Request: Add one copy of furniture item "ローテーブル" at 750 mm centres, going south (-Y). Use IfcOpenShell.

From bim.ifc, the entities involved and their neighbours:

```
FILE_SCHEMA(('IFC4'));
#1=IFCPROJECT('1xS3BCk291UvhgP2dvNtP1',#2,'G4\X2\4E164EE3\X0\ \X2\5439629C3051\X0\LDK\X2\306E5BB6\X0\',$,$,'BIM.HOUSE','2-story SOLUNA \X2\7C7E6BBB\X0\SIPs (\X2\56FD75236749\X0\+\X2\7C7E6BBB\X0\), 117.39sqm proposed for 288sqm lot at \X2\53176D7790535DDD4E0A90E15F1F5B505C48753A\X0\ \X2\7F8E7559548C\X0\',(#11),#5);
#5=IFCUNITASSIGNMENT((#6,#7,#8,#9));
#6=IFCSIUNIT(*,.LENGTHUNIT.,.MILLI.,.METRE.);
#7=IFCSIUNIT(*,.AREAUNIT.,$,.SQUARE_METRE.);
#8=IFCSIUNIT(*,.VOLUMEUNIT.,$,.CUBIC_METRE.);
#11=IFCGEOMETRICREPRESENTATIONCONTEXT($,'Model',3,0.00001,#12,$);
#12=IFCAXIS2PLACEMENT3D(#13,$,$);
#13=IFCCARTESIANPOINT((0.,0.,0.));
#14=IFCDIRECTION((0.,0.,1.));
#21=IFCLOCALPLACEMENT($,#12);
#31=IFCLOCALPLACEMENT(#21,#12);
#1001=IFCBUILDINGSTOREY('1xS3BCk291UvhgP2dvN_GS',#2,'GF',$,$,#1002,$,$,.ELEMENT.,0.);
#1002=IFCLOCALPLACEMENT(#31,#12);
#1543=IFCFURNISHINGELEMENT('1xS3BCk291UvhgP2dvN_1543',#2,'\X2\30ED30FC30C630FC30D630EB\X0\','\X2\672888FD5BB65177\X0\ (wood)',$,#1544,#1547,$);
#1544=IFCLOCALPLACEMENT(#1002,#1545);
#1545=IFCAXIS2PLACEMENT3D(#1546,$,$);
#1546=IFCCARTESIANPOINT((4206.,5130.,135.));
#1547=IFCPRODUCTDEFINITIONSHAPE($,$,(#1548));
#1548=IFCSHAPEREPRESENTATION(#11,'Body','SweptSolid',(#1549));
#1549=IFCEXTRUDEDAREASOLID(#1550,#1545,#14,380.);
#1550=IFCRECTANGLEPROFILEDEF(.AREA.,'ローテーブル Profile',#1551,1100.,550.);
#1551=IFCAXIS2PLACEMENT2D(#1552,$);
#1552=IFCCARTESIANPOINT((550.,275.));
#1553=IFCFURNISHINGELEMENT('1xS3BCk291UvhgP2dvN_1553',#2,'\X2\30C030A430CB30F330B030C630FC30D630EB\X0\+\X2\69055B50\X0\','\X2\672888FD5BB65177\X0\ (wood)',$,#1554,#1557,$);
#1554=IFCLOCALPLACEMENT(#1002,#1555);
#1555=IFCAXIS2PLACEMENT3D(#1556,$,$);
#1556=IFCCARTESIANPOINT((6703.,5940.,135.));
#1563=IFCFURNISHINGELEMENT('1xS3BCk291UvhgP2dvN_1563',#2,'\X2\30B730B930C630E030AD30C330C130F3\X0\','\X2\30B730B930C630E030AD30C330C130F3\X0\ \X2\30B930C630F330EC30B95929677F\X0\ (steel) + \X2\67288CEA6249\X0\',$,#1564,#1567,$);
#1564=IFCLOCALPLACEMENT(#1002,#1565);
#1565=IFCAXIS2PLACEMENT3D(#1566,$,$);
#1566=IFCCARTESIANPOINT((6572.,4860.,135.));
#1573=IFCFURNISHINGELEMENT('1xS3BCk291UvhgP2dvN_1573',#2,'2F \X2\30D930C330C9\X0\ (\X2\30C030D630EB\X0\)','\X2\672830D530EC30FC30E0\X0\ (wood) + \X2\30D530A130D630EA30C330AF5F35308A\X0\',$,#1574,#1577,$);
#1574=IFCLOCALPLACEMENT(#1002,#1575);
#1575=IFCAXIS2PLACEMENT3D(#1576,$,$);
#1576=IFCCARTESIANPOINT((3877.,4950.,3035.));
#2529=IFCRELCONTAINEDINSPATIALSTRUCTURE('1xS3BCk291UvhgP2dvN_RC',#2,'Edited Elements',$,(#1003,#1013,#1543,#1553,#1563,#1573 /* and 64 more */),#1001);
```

```python
import numpy as np
import ifcopenshell
import ifcopenshell.api.geometry
import ifcopenshell.api.root
import ifcopenshell.util.element
import ifcopenshell.util.placement
import ifcopenshell.util.unit

model = ifcopenshell.open("bim.ifc")
unit_scale = ifcopenshell.util.unit.calculate_unit_scale(model)


def reuse_history(source, copy):
    """copy_class also copies each property set's owner history, people and application; keep the originals."""
    for rel in copy.IsDefinedBy:
        if rel.is_a("IfcRelDefinesByProperties") and (history := rel.RelatingPropertyDefinition.OwnerHistory):
            rel.RelatingPropertyDefinition.OwnerHistory = source.OwnerHistory
            ifcopenshell.util.element.remove_deep2(model, history)


source = model.by_guid("1xS3BCk291UvhgP2dvN_1543")
base = ifcopenshell.util.placement.get_local_placement(source.ObjectPlacement)
step = np.array([0.0, -1.0, 0.0]) * 0.75 / unit_scale

for i in range(1, 2):
    copy = ifcopenshell.api.root.copy_class(model, product=source)
    copy.Representation = ifcopenshell.util.element.copy_deep(
        model, source.Representation, exclude=["IfcGeometricRepresentationContext", "IfcRepresentationMap"]
    )
    reuse_history(source, copy)
    matrix = base.copy()
    matrix[:3, 3] += i * step
    print("added at", matrix[:3, 3].round(3) + 0.0)
    ifcopenshell.api.geometry.edit_object_placement(model, product=copy, matrix=matrix, is_si=False)

model.write("bim-out.ifc")
```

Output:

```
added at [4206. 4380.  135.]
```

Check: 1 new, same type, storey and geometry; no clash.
